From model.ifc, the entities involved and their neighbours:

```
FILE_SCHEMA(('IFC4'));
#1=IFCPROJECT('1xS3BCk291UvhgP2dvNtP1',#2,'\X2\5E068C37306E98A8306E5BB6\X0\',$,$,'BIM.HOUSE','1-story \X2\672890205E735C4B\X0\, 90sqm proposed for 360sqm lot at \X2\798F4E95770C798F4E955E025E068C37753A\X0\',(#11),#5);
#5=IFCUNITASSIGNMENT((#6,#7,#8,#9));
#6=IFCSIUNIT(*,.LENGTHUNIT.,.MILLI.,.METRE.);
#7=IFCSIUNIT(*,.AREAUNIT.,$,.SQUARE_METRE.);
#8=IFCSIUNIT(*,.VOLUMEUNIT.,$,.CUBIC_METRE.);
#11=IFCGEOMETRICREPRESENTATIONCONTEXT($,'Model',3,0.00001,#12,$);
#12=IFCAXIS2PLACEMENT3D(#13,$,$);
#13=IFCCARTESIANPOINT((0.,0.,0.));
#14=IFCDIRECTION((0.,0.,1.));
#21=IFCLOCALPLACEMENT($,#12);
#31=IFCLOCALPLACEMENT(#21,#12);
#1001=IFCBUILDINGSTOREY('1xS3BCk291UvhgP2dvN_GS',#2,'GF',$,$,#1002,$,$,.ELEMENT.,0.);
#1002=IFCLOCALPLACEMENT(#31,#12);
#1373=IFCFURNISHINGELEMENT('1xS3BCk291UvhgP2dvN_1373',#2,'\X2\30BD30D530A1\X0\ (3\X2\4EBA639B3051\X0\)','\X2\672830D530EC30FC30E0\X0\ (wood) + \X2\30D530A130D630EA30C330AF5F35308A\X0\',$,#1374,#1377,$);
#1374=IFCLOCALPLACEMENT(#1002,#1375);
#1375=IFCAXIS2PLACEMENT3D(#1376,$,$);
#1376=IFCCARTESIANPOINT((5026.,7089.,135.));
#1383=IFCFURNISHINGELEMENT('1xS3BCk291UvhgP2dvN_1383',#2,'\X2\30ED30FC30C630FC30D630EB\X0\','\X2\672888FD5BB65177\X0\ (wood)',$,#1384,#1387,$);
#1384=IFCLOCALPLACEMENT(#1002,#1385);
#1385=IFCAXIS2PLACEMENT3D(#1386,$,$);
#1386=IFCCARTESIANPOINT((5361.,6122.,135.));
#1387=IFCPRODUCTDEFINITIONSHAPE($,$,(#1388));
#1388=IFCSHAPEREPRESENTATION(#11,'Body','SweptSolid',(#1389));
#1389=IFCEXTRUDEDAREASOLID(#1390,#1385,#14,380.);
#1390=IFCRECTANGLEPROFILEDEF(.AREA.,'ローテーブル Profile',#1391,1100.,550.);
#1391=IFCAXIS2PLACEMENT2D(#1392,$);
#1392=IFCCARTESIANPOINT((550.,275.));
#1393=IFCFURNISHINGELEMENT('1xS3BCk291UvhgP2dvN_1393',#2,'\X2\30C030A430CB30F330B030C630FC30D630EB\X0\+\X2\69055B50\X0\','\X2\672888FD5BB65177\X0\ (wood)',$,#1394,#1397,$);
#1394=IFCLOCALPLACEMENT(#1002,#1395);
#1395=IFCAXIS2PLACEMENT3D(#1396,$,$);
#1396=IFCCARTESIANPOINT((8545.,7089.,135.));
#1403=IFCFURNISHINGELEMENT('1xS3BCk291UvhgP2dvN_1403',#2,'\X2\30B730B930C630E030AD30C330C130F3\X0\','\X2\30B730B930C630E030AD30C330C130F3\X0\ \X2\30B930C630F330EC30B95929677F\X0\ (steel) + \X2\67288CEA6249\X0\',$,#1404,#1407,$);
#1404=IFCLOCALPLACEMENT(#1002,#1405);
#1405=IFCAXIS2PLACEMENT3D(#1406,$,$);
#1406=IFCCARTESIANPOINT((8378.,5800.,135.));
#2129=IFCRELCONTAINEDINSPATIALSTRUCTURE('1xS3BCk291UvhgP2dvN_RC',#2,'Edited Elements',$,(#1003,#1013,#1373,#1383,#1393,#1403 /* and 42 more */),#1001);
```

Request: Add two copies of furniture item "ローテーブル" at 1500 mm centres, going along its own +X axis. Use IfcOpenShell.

```python
import ifcopenshell
import ifcopenshell.api.geometry
import ifcopenshell.api.root
import ifcopenshell.util.element
import ifcopenshell.util.placement
import ifcopenshell.util.unit

model = ifcopenshell.open("model.ifc")
unit_scale = ifcopenshell.util.unit.calculate_unit_scale(model)


def reuse_history(source, copy):
    """copy_class also copies each property set's owner history, people and application; keep the originals."""
    for rel in copy.IsDefinedBy:
        if rel.is_a("IfcRelDefinesByProperties") and (history := rel.RelatingPropertyDefinition.OwnerHistory):
            rel.RelatingPropertyDefinition.OwnerHistory = source.OwnerHistory
            ifcopenshell.util.element.remove_deep2(model, history)


source = model.by_guid("1xS3BCk291UvhgP2dvN_1383")
base = ifcopenshell.util.placement.get_local_placement(source.ObjectPlacement)
step = base[:3, 0] * 1.5 / unit_scale

for i in range(1, 3):
    copy = ifcopenshell.api.root.copy_class(model, product=source)
    copy.Representation = ifcopenshell.util.element.copy_deep(
        model, source.Representation, exclude=["IfcGeometricRepresentationContext", "IfcRepresentationMap"]
    )
    reuse_history(source, copy)
    matrix = base.copy()
    matrix[:3, 3] += i * step
    print("added at", matrix[:3, 3].round(3) + 0.0)
    ifcopenshell.api.geometry.edit_object_placement(model, product=copy, matrix=matrix, is_si=False)

model.write("model-out.ifc")
```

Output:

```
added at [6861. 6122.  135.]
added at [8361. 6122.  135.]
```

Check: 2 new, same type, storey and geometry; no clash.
